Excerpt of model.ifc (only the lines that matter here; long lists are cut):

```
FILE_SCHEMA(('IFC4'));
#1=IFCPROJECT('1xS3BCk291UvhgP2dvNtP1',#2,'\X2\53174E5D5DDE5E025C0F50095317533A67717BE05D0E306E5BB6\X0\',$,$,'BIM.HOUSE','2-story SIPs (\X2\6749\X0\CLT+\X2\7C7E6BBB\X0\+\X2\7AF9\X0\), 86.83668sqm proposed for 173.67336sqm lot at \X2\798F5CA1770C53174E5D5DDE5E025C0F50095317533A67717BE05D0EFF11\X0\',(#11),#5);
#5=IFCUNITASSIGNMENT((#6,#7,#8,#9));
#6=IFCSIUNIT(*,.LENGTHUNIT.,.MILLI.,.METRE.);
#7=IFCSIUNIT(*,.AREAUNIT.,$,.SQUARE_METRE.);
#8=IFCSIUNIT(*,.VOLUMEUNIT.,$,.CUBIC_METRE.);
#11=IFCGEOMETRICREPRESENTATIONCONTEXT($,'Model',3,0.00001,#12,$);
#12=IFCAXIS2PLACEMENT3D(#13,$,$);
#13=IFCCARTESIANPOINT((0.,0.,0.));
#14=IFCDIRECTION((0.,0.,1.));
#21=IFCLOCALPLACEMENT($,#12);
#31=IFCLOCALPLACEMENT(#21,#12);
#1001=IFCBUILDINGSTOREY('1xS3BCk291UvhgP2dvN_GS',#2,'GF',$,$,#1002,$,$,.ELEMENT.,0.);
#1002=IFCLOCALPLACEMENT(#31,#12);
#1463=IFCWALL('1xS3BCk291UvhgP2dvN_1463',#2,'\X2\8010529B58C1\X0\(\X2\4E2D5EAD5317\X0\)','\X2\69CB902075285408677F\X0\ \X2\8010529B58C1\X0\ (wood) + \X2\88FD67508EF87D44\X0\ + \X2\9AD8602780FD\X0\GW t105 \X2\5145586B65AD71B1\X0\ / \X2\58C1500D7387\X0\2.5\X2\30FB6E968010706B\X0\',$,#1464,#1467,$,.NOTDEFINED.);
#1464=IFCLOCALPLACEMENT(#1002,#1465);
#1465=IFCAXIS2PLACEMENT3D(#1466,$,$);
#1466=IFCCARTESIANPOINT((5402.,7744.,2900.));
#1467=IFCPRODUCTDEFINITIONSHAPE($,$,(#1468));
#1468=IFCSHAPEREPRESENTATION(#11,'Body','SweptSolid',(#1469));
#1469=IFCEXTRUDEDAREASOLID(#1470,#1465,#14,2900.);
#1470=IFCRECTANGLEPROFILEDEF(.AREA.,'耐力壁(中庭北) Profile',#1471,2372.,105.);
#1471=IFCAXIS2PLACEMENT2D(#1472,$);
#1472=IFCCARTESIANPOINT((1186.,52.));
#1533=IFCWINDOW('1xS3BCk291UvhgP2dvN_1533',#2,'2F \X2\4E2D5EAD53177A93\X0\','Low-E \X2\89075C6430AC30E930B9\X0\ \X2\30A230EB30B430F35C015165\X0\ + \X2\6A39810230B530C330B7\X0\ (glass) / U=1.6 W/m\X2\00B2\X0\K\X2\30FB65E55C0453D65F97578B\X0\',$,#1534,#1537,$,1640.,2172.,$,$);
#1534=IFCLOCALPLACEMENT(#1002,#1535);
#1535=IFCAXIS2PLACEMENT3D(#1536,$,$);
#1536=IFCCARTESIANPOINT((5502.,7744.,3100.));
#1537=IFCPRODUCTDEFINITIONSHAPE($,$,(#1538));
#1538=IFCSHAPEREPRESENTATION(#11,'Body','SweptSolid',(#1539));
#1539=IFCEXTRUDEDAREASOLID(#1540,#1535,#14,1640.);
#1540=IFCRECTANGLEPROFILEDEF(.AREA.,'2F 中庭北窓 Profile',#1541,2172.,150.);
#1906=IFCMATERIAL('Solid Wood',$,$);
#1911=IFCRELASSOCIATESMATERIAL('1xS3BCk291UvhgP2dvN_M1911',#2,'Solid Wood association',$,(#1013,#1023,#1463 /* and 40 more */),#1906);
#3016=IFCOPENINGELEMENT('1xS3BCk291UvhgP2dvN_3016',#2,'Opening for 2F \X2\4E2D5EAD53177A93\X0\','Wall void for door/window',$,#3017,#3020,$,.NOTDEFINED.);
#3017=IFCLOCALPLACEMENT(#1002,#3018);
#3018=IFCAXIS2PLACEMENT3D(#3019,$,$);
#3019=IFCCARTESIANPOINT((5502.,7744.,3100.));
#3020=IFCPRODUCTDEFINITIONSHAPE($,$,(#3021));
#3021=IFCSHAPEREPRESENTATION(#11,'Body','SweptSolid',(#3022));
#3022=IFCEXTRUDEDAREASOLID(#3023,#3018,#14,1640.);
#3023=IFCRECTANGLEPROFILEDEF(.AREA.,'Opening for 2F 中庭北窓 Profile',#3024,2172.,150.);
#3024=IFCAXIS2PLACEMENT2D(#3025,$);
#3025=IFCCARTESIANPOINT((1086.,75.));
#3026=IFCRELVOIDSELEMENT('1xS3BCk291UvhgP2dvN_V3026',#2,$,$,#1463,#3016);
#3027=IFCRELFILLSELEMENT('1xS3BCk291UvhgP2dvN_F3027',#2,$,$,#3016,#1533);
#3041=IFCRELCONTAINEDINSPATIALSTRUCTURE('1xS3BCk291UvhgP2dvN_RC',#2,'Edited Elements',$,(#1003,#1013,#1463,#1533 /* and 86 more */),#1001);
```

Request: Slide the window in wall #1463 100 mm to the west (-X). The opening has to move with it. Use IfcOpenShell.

```python
import ifcopenshell
import ifcopenshell.api.geometry
import ifcopenshell.util.placement

model = ifcopenshell.open("model.ifc")

window = model.by_id(1533)
opening = window.FillsVoids[0].RelatingOpeningElement
wall = opening.VoidsElements[0].RelatingBuildingElement

wall_matrix = ifcopenshell.util.placement.get_local_placement(wall.ObjectPlacement)
shift = wall_matrix[:3, 0] * -100.0
before = ifcopenshell.util.placement.get_local_placement(window.ObjectPlacement)[:3, 3].copy()

# The window is not placed relative to its opening, so move both.
for product in (opening, window):
    matrix = ifcopenshell.util.placement.get_local_placement(product.ObjectPlacement)
    matrix[:3, 3] += shift
    ifcopenshell.api.geometry.edit_object_placement(model, product=product, matrix=matrix, is_si=False)

after = ifcopenshell.util.placement.get_local_placement(window.ObjectPlacement)[:3, 3]
print("window moved by", (after - before).round(3) + 0.0)

model.write("model_updated.ifc")
```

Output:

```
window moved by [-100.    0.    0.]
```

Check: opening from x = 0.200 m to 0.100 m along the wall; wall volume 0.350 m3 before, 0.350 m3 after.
